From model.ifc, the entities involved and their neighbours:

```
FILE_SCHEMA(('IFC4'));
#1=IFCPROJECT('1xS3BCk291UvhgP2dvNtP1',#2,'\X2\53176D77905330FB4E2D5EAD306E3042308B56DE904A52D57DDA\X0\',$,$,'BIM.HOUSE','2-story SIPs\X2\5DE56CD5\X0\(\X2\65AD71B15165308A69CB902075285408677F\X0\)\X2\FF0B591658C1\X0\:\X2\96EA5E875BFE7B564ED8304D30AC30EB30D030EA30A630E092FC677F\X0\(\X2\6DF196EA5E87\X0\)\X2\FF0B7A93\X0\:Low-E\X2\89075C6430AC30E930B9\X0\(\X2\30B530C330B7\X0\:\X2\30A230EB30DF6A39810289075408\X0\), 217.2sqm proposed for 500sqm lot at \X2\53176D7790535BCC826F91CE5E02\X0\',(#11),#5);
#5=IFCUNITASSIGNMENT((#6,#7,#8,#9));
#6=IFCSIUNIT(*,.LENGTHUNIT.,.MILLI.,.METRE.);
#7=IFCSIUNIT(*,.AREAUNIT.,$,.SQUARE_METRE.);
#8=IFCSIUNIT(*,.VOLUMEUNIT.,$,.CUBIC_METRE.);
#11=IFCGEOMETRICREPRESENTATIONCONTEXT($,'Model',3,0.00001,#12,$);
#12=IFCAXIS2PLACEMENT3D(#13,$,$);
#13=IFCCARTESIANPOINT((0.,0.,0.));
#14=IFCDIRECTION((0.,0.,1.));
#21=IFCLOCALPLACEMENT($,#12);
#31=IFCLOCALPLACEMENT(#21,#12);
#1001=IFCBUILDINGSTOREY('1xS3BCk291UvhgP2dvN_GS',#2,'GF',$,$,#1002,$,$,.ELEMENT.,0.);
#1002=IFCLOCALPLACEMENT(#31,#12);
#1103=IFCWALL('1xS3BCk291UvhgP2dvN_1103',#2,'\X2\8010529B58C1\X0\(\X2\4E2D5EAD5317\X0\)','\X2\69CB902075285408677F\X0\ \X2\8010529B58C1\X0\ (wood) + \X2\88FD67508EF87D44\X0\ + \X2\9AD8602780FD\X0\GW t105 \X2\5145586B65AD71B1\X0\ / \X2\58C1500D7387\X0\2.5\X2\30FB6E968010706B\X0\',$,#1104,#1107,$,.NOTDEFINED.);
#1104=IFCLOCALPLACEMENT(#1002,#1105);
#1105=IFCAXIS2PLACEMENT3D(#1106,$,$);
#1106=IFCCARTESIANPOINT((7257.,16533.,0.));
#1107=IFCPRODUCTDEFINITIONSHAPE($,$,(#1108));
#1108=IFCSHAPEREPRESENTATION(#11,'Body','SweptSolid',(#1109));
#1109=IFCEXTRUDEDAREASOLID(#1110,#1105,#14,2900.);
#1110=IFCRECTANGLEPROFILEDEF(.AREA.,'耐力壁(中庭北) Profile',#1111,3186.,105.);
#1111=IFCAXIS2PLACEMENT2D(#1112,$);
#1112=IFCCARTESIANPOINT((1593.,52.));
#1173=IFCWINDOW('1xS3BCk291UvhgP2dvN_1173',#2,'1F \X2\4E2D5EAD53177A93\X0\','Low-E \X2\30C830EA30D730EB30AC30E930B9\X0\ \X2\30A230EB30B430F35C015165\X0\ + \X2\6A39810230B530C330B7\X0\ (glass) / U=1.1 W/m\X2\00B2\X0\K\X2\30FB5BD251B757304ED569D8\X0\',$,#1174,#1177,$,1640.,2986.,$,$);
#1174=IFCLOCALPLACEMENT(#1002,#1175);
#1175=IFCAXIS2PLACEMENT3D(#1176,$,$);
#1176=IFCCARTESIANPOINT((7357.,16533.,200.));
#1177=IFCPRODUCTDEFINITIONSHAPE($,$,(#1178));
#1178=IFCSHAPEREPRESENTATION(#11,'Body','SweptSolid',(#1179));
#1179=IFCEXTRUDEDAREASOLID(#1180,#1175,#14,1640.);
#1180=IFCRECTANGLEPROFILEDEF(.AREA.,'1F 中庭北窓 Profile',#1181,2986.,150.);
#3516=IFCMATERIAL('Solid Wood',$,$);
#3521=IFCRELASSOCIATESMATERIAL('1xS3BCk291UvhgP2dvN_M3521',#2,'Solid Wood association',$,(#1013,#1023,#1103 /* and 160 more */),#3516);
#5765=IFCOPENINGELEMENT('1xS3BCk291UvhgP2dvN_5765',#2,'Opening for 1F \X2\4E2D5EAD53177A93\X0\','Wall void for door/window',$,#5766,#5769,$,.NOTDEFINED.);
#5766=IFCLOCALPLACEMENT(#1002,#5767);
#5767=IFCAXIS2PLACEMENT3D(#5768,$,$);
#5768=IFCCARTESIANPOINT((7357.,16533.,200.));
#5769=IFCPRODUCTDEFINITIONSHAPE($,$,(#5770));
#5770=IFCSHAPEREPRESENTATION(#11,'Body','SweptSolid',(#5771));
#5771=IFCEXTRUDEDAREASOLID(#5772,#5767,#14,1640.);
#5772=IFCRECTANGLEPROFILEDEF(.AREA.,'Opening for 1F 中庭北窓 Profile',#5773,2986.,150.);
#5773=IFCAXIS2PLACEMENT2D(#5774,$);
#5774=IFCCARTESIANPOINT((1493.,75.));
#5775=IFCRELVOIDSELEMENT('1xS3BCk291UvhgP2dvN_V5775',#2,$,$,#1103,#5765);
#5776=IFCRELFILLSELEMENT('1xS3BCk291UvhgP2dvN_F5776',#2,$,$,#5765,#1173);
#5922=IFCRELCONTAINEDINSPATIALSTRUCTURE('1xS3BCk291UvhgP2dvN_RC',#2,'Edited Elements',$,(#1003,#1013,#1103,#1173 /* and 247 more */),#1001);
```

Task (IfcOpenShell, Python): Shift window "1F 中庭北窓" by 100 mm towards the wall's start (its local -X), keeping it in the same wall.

```python
import ifcopenshell
import ifcopenshell.api.geometry
import ifcopenshell.util.placement

model = ifcopenshell.open("model.ifc")

window = model.by_guid("1xS3BCk291UvhgP2dvN_1173")
opening = window.FillsVoids[0].RelatingOpeningElement
wall = opening.VoidsElements[0].RelatingBuildingElement

wall_matrix = ifcopenshell.util.placement.get_local_placement(wall.ObjectPlacement)
shift = wall_matrix[:3, 0] * -100.0
before = ifcopenshell.util.placement.get_local_placement(window.ObjectPlacement)[:3, 3].copy()

# The window is not placed relative to its opening, so move both.
for product in (opening, window):
    matrix = ifcopenshell.util.placement.get_local_placement(product.ObjectPlacement)
    matrix[:3, 3] += shift
    ifcopenshell.api.geometry.edit_object_placement(model, product=product, matrix=matrix, is_si=False)

after = ifcopenshell.util.placement.get_local_placement(window.ObjectPlacement)[:3, 3]
print("window moved by", (after - before).round(3) + 0.0)

model.write("model_updated.ifc")
```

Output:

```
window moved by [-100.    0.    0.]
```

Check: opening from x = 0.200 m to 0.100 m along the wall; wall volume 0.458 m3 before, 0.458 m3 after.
